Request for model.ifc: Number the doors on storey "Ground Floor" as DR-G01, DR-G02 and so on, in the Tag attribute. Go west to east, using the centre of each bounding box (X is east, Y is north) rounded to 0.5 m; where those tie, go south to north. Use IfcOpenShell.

First a look at what the model holds.

```python
import ifcopenshell
import ifcopenshell.util.element
import ifcopenshell.util.placement

model = ifcopenshell.open("model.ifc")
print(model.schema)
storey = next(s for s in model.by_type("IfcBuildingStorey") if s.Name == "Ground Floor")
doors = [e for e in ifcopenshell.util.element.get_decomposition(storey) if e.is_a("IfcDoor")]
for e in sorted(doors, key=lambda e: e.id()):
    origin = ifcopenshell.util.placement.get_local_placement(e.ObjectPlacement)[:3, 3]
    print(e.id(), e.Tag, e.Name, origin.round(2) + 0.0, sep=" | ")
```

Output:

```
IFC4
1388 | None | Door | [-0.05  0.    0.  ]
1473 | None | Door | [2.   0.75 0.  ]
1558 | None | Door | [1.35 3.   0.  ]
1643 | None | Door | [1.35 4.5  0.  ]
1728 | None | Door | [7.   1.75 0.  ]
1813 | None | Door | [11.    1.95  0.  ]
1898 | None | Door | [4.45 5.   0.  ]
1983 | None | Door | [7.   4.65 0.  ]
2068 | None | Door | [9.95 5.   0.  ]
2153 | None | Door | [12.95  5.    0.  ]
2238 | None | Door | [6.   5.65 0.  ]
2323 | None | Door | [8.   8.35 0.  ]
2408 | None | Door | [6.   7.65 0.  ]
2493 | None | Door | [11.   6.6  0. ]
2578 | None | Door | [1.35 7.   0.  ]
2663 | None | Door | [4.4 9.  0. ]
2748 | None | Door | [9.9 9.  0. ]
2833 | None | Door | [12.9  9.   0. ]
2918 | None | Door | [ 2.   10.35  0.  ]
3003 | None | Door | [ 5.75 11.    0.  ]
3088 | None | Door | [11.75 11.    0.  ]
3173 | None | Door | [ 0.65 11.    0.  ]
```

```python
import ifcopenshell
import ifcopenshell.geom
import ifcopenshell.util.element
import ifcopenshell.util.shape

model = ifcopenshell.open("model.ifc")
settings = ifcopenshell.geom.settings()
settings.set("use-world-coords", True)


def centre(element):
    shape = ifcopenshell.geom.create_shape(settings, element)
    return ifcopenshell.util.shape.get_bbox_centroid(shape.geometry)


storey = next(s for s in model.by_type("IfcBuildingStorey") if s.Name == "Ground Floor")
doors = [e for e in ifcopenshell.util.element.get_decomposition(storey) if e.is_a("IfcDoor")]

# Insertion points can sit at a corner or the storey origin, so sort by the geometry (in metres).
centres = {e: centre(e) for e in doors}
doors.sort(key=lambda e: (round(centres[e][0] / 0.5), centres[e][1]))

for i, e in enumerate(doors, start=1):
    number = f"DR-G{i:02d}"
    e.Tag = number
    print(e.id(), number)

model.write("model_v2.ifc")
```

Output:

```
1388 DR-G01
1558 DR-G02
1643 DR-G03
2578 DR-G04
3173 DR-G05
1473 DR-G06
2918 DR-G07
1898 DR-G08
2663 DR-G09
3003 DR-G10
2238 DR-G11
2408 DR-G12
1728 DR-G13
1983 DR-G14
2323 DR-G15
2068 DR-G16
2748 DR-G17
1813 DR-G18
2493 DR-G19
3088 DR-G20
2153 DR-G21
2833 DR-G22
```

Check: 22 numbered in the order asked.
